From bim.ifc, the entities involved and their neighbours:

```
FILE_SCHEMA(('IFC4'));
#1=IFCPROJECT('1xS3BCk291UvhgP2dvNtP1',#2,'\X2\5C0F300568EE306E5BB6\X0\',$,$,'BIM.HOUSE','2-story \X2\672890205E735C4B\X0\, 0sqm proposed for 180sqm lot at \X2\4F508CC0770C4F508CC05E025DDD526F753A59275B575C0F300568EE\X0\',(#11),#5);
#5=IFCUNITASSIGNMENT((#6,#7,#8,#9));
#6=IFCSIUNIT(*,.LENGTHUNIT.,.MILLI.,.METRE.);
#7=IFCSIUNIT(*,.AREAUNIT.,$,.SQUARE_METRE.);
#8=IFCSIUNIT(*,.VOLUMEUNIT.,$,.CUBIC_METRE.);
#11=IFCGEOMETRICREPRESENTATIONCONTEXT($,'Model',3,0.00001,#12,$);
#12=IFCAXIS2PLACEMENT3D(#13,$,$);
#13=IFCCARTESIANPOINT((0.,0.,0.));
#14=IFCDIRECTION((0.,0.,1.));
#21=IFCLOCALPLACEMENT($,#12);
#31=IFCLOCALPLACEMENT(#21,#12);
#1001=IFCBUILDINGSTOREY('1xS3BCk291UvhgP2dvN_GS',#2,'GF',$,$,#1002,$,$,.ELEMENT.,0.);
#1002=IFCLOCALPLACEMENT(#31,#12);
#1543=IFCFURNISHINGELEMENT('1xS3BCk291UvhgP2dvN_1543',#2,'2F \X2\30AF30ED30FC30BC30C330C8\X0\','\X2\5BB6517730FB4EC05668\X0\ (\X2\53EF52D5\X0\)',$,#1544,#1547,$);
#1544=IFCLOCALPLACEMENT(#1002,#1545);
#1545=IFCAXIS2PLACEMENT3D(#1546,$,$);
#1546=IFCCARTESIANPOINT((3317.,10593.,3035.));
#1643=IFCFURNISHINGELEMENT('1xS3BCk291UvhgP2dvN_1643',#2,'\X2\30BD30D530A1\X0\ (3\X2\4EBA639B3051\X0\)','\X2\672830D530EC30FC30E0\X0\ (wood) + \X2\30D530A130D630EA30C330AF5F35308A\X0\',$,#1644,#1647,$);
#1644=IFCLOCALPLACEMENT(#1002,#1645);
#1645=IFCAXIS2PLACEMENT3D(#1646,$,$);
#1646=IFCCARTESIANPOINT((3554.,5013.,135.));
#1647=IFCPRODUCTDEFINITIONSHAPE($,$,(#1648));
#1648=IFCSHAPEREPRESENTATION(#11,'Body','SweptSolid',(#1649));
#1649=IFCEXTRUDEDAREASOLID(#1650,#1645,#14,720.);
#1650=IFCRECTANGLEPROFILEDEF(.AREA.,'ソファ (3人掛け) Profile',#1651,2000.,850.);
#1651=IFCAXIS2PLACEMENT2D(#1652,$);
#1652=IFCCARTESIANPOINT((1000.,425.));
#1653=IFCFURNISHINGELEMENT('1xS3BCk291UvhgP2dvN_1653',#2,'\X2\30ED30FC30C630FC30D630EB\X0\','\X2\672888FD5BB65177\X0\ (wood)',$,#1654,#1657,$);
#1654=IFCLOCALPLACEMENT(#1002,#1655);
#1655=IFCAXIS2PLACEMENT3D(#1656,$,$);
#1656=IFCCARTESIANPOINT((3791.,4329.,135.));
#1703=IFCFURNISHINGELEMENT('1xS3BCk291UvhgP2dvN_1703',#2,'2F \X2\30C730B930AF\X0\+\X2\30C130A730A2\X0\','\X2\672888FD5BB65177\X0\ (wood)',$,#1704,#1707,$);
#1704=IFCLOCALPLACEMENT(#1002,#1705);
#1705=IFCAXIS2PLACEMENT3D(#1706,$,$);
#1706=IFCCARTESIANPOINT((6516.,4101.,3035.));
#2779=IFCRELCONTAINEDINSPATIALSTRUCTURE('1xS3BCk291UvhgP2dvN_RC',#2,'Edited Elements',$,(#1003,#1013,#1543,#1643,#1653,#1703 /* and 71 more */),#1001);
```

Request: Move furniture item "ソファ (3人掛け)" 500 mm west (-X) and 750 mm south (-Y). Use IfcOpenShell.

```python
import ifcopenshell
import ifcopenshell.api.geometry
import ifcopenshell.util.placement
import ifcopenshell.util.unit

model = ifcopenshell.open("bim.ifc")
unit_scale = ifcopenshell.util.unit.calculate_unit_scale(model)

item = model.by_guid("1xS3BCk291UvhgP2dvN_1643")
matrix = ifcopenshell.util.placement.get_local_placement(item.ObjectPlacement)
matrix[0, 3] -= 0.5 / unit_scale
matrix[1, 3] -= 0.75 / unit_scale
ifcopenshell.api.geometry.edit_object_placement(model, product=item, matrix=matrix, is_si=False)

print(ifcopenshell.util.placement.get_local_placement(item.ObjectPlacement).round(3) + 0.0)

model.write("bim_edited.ifc")
```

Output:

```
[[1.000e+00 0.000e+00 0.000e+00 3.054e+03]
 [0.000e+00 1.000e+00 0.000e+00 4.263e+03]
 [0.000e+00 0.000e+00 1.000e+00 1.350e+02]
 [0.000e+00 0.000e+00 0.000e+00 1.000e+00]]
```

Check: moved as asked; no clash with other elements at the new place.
